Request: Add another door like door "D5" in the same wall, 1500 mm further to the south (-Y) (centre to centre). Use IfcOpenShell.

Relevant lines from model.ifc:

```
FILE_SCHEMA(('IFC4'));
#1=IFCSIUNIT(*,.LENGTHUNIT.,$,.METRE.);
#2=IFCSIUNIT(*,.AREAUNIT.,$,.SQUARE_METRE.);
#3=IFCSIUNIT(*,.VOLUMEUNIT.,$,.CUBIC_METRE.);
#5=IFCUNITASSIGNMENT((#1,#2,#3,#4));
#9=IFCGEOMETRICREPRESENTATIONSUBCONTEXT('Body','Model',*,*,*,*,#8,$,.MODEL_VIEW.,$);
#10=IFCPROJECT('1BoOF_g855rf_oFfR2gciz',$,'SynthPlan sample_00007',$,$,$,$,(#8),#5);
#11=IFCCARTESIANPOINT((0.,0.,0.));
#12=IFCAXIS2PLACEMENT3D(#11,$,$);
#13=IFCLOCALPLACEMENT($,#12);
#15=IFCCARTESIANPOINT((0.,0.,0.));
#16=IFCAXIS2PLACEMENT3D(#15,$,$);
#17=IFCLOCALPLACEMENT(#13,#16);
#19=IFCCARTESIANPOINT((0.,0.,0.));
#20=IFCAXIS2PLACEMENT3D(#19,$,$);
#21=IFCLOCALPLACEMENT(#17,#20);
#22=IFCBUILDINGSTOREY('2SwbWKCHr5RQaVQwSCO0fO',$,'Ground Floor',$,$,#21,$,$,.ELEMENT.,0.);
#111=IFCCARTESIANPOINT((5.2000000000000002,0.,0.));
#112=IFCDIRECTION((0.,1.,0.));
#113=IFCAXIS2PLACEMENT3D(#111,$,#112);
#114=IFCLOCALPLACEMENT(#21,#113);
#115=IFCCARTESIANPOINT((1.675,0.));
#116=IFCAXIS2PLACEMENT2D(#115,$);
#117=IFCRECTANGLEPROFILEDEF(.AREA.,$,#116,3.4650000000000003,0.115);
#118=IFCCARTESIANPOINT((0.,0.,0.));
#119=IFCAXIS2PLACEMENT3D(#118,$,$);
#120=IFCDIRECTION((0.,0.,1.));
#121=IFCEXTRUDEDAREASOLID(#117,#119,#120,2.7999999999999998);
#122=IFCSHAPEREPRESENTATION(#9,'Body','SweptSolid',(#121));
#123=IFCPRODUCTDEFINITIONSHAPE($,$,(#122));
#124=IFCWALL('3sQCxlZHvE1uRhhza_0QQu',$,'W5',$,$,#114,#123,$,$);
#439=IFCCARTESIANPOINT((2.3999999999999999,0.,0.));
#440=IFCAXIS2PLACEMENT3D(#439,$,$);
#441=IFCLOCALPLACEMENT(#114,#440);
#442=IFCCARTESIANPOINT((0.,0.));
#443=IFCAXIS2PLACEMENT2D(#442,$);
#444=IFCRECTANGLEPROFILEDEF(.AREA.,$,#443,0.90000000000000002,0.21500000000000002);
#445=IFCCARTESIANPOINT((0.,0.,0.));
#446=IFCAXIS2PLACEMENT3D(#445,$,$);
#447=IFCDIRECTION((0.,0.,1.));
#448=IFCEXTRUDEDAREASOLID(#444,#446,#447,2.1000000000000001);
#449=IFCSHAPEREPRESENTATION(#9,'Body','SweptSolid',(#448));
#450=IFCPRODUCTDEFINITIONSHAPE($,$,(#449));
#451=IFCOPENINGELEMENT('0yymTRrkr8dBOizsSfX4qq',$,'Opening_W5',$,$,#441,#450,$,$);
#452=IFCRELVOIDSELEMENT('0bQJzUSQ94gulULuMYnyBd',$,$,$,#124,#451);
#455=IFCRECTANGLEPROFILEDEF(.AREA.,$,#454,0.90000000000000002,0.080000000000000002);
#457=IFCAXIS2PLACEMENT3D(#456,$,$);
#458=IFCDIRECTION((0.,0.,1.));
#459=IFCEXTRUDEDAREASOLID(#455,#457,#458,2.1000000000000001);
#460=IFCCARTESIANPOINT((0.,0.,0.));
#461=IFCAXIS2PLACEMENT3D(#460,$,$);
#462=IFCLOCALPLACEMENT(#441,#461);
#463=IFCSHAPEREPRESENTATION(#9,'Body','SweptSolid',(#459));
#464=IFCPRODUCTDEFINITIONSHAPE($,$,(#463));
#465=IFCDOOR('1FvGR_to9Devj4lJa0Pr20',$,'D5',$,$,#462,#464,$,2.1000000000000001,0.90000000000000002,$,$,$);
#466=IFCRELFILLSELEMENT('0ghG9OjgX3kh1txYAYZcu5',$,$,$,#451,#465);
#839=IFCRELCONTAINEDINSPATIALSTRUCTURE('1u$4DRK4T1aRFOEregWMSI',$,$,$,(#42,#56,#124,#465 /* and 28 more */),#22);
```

```python
import ifcopenshell
import ifcopenshell.api.feature
import ifcopenshell.api.geometry
import ifcopenshell.api.root
import ifcopenshell.geom
import ifcopenshell.util.element
import ifcopenshell.util.placement
import ifcopenshell.util.shape
import ifcopenshell.util.unit

model = ifcopenshell.open("model.ifc")
unit_scale = ifcopenshell.util.unit.calculate_unit_scale(model)
settings = ifcopenshell.geom.settings()


def volume(element):
    """Net volume in cubic metres, openings subtracted."""
    shape = ifcopenshell.geom.create_shape(settings, element)
    return ifcopenshell.util.shape.get_volume(shape.geometry)


door = model.by_guid("1FvGR_to9Devj4lJa0Pr20")
opening = door.FillsVoids[0].RelatingOpeningElement
wall = opening.VoidsElements[0].RelatingBuildingElement
before = volume(wall)
shift = ifcopenshell.util.placement.get_local_placement(wall.ObjectPlacement)[:3, 0] * -1.5 / unit_scale

# copy_class copies the void relationship, type, container and properties, but no geometry.
new_opening = ifcopenshell.api.root.copy_class(model, product=opening)
new_opening.Representation = ifcopenshell.util.element.copy_deep(
    model, opening.Representation, exclude=["IfcGeometricRepresentationContext", "IfcRepresentationMap"]
)
new_door = ifcopenshell.api.root.copy_class(model, product=door)
new_door.Representation = ifcopenshell.util.element.copy_deep(
    model, door.Representation, exclude=["IfcGeometricRepresentationContext", "IfcRepresentationMap"]
)
ifcopenshell.api.feature.add_filling(model, opening=new_opening, element=new_door)

for old, new in ((opening, new_opening), (door, new_door)):
    matrix = ifcopenshell.util.placement.get_local_placement(old.ObjectPlacement)
    matrix[:3, 3] += shift
    ifcopenshell.api.geometry.edit_object_placement(model, product=new, matrix=matrix, is_si=False)

after = volume(wall)

print(f"wall volume {before:.3f} -> {after:.3f} m3")

model.write("model_rev.ifc")
```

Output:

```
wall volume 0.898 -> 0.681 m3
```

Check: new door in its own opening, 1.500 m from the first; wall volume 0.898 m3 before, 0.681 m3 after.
